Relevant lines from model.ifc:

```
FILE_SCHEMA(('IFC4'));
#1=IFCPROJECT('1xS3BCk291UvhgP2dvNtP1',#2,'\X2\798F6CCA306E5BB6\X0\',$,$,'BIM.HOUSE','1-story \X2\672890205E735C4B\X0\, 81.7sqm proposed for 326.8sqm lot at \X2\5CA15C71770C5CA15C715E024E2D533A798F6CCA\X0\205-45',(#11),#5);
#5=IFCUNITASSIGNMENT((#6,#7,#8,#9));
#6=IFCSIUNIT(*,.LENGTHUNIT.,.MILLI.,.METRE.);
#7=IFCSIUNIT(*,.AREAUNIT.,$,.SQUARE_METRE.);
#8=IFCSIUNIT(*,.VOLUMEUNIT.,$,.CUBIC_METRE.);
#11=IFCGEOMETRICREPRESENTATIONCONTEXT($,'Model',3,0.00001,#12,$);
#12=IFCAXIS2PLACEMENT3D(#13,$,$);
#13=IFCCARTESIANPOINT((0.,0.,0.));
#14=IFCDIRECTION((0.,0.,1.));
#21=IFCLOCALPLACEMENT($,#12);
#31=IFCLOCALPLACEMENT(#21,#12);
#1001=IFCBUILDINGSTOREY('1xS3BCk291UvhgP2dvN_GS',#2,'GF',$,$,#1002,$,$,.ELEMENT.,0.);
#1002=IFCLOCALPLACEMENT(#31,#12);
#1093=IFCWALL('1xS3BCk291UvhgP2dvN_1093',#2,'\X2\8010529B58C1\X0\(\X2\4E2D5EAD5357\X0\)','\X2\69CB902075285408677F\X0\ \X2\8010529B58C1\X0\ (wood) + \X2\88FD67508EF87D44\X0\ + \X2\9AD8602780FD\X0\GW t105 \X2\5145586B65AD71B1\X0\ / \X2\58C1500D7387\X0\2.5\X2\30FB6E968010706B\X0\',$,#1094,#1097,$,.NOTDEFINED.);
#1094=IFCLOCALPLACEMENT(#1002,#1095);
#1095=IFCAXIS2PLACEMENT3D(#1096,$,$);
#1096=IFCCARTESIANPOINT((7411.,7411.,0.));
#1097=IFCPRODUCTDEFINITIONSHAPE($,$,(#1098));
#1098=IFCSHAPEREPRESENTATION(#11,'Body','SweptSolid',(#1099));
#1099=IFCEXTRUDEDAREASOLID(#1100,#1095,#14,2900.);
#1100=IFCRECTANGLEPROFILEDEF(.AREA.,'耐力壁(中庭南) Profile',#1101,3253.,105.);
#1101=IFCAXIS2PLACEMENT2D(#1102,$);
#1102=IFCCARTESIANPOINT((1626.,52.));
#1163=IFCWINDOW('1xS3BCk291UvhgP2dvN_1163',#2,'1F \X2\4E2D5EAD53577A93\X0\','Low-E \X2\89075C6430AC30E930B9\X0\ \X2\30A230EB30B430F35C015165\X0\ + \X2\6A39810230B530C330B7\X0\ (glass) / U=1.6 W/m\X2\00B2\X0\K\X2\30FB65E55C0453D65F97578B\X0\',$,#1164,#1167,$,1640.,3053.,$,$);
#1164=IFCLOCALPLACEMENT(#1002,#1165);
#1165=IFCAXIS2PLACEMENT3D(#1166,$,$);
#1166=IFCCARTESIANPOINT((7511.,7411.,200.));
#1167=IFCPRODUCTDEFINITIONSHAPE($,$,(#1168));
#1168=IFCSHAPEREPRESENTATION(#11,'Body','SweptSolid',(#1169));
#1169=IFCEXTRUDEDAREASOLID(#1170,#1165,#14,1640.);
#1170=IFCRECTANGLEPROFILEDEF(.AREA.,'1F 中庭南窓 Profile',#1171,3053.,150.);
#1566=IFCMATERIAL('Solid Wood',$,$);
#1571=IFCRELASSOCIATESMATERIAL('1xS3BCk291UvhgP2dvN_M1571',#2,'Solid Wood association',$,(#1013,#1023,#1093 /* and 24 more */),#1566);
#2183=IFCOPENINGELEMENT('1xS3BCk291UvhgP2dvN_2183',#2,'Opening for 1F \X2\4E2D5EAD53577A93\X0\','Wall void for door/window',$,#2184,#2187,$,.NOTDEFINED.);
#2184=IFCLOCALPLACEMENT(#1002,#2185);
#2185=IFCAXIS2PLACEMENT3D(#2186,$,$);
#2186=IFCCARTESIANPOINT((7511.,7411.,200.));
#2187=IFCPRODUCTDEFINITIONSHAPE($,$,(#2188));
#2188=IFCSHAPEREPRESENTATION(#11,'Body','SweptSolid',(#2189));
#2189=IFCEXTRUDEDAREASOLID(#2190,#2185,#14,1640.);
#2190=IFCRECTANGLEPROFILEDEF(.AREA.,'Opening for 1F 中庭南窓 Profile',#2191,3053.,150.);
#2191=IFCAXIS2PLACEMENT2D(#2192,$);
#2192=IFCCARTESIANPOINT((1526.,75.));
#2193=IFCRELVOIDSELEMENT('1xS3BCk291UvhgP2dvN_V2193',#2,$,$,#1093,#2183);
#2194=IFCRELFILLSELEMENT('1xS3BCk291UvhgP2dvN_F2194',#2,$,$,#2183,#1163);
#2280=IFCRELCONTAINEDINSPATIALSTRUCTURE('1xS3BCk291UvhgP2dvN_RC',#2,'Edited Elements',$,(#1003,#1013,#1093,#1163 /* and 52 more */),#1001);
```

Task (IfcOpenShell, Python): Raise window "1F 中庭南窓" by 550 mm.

```python
import numpy as np
import ifcopenshell
import ifcopenshell.api.geometry
import ifcopenshell.util.placement
import ifcopenshell.util.unit

model = ifcopenshell.open("model.ifc")
unit_scale = ifcopenshell.util.unit.calculate_unit_scale(model)

window = model.by_guid("1xS3BCk291UvhgP2dvN_1163")
opening = window.FillsVoids[0].RelatingOpeningElement
dz = 550.0

shift = np.array([0.0, 0.0, dz])
# The window is not placed relative to its opening, so move both.
for product in (opening, window):
    matrix = ifcopenshell.util.placement.get_local_placement(product.ObjectPlacement)
    matrix[:3, 3] += shift
    ifcopenshell.api.geometry.edit_object_placement(model, product=product, matrix=matrix, is_si=False)

print(f"moved by {dz * unit_scale:+.3f} m")

model.write("model_updated.ifc")
```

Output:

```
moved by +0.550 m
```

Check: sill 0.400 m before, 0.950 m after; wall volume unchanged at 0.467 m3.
